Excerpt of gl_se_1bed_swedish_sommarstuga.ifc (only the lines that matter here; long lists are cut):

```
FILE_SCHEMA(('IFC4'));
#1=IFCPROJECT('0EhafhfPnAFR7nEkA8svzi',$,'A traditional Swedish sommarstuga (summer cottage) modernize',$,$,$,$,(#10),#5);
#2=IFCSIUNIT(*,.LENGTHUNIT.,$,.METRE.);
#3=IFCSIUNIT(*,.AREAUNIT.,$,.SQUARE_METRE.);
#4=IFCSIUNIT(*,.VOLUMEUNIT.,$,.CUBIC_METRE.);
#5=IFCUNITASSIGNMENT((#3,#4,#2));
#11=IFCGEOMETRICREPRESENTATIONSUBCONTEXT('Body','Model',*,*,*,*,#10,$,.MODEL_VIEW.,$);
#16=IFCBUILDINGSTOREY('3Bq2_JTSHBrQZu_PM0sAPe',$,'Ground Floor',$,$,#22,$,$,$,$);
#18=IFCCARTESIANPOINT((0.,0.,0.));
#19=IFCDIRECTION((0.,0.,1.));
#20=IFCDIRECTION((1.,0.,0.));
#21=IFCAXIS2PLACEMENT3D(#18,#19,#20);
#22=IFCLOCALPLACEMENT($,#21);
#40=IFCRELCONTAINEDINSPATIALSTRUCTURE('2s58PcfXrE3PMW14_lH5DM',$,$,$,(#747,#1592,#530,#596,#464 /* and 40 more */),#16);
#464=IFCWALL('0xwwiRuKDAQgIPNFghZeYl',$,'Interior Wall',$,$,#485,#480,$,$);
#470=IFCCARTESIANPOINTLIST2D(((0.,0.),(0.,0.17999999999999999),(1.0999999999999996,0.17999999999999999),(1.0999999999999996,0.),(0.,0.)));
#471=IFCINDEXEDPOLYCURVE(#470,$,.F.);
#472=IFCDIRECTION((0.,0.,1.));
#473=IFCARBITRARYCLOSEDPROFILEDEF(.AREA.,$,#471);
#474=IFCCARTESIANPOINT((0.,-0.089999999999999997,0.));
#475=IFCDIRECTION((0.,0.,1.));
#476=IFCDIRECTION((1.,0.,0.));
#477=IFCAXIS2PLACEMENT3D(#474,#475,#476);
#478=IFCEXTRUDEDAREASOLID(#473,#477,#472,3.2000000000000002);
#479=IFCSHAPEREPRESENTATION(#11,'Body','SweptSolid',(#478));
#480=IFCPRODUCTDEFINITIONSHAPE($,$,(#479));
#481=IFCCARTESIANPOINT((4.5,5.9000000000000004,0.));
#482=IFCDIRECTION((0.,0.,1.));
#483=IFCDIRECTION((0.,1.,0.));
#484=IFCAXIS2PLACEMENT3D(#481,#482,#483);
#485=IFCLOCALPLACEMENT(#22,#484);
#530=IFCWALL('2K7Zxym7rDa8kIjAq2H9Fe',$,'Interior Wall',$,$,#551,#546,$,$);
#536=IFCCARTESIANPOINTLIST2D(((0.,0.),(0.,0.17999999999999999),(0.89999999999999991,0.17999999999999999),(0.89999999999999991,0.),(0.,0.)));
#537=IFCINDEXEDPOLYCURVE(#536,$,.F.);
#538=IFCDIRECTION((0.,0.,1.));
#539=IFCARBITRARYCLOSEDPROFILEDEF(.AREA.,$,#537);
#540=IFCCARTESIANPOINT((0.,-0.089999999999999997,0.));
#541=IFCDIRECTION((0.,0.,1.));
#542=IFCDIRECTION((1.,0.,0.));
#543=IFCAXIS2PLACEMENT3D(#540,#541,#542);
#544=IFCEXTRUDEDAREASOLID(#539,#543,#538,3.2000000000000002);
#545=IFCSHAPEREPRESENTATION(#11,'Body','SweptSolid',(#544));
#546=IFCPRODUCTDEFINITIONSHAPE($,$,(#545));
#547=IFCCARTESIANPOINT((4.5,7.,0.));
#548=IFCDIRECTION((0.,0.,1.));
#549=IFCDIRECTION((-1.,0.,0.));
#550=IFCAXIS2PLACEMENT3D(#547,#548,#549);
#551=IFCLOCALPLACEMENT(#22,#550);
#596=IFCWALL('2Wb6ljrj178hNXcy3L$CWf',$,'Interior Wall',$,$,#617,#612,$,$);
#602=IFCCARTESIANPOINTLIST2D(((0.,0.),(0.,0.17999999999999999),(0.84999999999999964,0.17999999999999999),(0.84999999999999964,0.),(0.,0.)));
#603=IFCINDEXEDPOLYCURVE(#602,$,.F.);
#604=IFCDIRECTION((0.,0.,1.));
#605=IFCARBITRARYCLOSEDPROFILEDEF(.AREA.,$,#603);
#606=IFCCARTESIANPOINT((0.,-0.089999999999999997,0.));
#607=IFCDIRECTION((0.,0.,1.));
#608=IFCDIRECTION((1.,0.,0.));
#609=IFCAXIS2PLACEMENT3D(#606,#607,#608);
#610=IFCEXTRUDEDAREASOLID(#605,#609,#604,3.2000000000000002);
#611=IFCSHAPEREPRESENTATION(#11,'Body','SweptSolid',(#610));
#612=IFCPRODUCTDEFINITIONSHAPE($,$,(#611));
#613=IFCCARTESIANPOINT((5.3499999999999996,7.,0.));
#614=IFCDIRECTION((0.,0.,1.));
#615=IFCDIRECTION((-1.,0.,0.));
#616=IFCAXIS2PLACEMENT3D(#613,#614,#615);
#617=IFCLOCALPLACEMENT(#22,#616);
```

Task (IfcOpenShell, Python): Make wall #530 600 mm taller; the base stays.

```python
import ifcopenshell
import ifcopenshell.geom
import ifcopenshell.util.representation
import ifcopenshell.util.shape

model = ifcopenshell.open("gl_se_1bed_swedish_sommarstuga.ifc")
settings = ifcopenshell.geom.settings()


def volume(element):
    """Net volume in cubic metres, openings subtracted."""
    shape = ifcopenshell.geom.create_shape(settings, element)
    return ifcopenshell.util.shape.get_volume(shape.geometry)


wall = model.by_guid("2K7Zxym7rDa8kIjAq2H9Fe")
before = volume(wall)

body = ifcopenshell.util.representation.get_representation(wall, "Model", "Body")
solid = body.Items[0]
old_height = solid.Depth
solid.Depth += 0.6
after = volume(wall)

print(f"height {old_height:g} -> {solid.Depth:g}, volume {before:.3f} -> {after:.3f} m3")

model.write("gl_se_1bed_swedish_sommarstuga_edited.ifc")
```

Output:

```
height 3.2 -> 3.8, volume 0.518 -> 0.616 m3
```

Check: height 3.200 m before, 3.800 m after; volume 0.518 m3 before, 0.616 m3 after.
